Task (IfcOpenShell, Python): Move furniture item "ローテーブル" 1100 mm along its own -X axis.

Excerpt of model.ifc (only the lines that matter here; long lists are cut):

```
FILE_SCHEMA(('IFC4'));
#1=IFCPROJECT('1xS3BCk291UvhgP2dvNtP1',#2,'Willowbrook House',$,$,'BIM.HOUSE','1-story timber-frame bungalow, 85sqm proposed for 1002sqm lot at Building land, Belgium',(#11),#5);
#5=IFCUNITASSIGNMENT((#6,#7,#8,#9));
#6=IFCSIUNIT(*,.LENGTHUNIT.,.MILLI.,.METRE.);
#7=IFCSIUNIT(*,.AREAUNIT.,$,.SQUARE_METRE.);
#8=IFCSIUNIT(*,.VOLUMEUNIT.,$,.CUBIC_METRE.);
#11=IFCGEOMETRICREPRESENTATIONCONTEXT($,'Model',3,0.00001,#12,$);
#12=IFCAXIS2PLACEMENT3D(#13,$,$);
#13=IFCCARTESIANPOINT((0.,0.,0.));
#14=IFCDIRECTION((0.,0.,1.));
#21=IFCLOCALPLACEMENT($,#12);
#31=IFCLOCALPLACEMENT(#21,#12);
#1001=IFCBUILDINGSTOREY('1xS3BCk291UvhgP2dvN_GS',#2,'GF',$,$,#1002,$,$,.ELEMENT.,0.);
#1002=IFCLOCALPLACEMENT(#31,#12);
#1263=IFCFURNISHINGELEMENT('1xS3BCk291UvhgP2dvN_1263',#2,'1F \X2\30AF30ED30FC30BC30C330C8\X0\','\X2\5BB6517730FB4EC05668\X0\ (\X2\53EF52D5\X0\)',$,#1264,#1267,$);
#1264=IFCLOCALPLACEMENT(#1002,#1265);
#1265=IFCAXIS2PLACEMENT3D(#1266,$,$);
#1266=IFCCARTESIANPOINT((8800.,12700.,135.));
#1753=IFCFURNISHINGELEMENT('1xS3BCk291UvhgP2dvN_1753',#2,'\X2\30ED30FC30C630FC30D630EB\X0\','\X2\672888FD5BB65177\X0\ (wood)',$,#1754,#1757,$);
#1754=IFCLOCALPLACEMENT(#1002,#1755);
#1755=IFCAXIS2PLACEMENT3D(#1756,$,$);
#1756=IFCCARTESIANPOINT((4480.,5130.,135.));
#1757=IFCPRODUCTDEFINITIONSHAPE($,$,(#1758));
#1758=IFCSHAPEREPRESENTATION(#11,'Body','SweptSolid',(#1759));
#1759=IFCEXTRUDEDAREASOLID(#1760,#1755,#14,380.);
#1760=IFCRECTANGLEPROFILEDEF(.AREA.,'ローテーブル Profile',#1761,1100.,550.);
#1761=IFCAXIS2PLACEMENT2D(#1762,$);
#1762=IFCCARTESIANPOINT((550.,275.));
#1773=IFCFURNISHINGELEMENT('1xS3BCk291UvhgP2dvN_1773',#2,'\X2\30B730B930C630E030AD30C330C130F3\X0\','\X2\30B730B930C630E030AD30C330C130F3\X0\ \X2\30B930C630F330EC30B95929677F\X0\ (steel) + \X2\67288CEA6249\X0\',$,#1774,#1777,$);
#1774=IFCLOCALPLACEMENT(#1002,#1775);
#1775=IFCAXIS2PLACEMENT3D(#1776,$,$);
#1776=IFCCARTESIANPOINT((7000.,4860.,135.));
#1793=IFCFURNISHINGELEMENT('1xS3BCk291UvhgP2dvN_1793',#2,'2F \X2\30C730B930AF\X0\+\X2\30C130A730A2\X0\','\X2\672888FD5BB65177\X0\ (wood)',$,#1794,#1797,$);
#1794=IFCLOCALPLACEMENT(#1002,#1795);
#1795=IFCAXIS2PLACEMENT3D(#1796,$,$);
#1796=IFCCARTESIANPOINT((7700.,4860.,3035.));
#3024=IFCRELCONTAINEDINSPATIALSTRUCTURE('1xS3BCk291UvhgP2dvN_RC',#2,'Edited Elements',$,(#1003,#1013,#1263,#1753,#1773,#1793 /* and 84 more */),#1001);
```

```python
import ifcopenshell
import ifcopenshell.api.geometry
import ifcopenshell.util.placement
import ifcopenshell.util.unit

model = ifcopenshell.open("model.ifc")
unit_scale = ifcopenshell.util.unit.calculate_unit_scale(model)

item = model.by_guid("1xS3BCk291UvhgP2dvN_1753")
matrix = ifcopenshell.util.placement.get_local_placement(item.ObjectPlacement)
matrix[:3, 3] -= matrix[:3, 0] * 1.1 / unit_scale
ifcopenshell.api.geometry.edit_object_placement(model, product=item, matrix=matrix, is_si=False)

print(ifcopenshell.util.placement.get_local_placement(item.ObjectPlacement).round(3) + 0.0)

model.write("model_rev.ifc")
```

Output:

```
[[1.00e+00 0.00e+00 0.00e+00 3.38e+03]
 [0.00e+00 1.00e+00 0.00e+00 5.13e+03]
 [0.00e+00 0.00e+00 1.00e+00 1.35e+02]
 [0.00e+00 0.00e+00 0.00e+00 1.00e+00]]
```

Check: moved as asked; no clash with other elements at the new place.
